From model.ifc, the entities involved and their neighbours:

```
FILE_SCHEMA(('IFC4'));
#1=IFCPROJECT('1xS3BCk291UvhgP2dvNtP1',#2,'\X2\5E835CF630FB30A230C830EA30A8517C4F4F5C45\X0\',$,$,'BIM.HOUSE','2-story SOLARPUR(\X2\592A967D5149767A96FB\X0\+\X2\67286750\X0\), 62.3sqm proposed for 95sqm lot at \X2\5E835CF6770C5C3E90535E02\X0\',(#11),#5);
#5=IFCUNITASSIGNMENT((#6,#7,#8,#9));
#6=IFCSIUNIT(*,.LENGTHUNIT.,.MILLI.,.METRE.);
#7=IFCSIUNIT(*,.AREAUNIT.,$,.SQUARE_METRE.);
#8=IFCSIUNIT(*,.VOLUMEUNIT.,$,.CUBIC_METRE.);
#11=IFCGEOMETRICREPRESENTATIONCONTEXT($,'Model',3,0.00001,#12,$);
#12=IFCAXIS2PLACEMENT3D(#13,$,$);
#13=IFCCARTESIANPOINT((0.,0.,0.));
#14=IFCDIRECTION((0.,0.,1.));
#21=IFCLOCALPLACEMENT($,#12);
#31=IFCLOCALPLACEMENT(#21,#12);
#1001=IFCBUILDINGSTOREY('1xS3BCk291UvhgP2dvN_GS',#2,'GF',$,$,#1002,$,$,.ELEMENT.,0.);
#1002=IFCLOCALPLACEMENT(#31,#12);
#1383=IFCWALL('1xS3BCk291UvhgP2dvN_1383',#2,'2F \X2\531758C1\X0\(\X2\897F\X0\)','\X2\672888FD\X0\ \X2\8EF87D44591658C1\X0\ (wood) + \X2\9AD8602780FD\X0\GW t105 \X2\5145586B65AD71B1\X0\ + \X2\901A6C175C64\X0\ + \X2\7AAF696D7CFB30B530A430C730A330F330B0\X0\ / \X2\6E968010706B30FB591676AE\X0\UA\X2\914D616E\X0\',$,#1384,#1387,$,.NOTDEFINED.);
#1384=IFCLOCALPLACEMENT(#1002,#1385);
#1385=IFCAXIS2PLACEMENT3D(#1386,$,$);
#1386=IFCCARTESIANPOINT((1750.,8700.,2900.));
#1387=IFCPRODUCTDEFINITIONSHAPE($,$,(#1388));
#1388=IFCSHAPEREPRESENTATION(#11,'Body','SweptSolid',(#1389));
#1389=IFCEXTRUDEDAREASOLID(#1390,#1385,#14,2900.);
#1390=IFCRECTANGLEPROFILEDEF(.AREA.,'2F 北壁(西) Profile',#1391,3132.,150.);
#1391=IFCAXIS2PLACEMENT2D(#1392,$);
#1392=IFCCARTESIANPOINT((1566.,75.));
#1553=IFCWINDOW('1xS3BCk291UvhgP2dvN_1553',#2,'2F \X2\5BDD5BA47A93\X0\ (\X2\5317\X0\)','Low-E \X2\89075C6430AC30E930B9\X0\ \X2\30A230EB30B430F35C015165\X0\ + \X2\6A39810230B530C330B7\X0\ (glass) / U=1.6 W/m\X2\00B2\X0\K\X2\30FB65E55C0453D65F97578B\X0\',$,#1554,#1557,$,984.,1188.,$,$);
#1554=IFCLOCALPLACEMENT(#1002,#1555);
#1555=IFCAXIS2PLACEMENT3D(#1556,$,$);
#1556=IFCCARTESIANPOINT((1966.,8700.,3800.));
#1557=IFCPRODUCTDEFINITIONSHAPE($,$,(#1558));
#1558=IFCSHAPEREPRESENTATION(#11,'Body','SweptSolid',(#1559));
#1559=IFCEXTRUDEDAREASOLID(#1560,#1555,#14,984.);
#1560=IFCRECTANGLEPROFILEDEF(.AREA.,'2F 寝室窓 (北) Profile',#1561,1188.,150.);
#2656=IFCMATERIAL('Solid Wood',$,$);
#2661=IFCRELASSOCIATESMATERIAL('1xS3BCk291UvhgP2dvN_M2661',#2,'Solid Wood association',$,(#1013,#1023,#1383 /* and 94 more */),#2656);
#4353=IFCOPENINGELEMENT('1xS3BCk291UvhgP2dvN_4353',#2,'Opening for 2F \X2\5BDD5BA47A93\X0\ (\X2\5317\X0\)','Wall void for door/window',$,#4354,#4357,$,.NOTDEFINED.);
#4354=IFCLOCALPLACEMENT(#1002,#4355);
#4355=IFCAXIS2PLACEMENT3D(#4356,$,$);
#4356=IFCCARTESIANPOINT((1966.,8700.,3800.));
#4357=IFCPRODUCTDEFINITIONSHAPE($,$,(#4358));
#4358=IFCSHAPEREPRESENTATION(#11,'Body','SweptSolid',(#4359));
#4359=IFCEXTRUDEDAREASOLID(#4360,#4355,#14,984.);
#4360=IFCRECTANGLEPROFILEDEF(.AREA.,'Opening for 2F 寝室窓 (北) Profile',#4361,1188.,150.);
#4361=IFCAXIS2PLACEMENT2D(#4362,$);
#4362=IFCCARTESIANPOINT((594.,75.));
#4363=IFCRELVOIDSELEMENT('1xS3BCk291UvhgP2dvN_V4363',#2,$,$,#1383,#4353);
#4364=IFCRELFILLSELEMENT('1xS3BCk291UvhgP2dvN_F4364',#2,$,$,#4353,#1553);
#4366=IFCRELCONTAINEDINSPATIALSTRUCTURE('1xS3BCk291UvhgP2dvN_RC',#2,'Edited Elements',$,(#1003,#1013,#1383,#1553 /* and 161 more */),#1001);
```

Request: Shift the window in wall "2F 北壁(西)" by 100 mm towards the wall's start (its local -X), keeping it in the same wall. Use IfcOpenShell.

```python
import ifcopenshell
import ifcopenshell.api.geometry
import ifcopenshell.util.placement

model = ifcopenshell.open("model.ifc")

window = model.by_guid("1xS3BCk291UvhgP2dvN_1553")
opening = window.FillsVoids[0].RelatingOpeningElement
wall = opening.VoidsElements[0].RelatingBuildingElement

wall_matrix = ifcopenshell.util.placement.get_local_placement(wall.ObjectPlacement)
shift = wall_matrix[:3, 0] * -100.0
before = ifcopenshell.util.placement.get_local_placement(window.ObjectPlacement)[:3, 3].copy()

# The window is not placed relative to its opening, so move both.
for product in (opening, window):
    matrix = ifcopenshell.util.placement.get_local_placement(product.ObjectPlacement)
    matrix[:3, 3] += shift
    ifcopenshell.api.geometry.edit_object_placement(model, product=product, matrix=matrix, is_si=False)

after = ifcopenshell.util.placement.get_local_placement(window.ObjectPlacement)[:3, 3]
print("window moved by", (after - before).round(3) + 0.0)

model.write("model_edited.ifc")
```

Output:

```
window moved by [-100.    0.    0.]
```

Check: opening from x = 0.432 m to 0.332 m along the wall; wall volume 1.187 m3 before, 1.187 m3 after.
